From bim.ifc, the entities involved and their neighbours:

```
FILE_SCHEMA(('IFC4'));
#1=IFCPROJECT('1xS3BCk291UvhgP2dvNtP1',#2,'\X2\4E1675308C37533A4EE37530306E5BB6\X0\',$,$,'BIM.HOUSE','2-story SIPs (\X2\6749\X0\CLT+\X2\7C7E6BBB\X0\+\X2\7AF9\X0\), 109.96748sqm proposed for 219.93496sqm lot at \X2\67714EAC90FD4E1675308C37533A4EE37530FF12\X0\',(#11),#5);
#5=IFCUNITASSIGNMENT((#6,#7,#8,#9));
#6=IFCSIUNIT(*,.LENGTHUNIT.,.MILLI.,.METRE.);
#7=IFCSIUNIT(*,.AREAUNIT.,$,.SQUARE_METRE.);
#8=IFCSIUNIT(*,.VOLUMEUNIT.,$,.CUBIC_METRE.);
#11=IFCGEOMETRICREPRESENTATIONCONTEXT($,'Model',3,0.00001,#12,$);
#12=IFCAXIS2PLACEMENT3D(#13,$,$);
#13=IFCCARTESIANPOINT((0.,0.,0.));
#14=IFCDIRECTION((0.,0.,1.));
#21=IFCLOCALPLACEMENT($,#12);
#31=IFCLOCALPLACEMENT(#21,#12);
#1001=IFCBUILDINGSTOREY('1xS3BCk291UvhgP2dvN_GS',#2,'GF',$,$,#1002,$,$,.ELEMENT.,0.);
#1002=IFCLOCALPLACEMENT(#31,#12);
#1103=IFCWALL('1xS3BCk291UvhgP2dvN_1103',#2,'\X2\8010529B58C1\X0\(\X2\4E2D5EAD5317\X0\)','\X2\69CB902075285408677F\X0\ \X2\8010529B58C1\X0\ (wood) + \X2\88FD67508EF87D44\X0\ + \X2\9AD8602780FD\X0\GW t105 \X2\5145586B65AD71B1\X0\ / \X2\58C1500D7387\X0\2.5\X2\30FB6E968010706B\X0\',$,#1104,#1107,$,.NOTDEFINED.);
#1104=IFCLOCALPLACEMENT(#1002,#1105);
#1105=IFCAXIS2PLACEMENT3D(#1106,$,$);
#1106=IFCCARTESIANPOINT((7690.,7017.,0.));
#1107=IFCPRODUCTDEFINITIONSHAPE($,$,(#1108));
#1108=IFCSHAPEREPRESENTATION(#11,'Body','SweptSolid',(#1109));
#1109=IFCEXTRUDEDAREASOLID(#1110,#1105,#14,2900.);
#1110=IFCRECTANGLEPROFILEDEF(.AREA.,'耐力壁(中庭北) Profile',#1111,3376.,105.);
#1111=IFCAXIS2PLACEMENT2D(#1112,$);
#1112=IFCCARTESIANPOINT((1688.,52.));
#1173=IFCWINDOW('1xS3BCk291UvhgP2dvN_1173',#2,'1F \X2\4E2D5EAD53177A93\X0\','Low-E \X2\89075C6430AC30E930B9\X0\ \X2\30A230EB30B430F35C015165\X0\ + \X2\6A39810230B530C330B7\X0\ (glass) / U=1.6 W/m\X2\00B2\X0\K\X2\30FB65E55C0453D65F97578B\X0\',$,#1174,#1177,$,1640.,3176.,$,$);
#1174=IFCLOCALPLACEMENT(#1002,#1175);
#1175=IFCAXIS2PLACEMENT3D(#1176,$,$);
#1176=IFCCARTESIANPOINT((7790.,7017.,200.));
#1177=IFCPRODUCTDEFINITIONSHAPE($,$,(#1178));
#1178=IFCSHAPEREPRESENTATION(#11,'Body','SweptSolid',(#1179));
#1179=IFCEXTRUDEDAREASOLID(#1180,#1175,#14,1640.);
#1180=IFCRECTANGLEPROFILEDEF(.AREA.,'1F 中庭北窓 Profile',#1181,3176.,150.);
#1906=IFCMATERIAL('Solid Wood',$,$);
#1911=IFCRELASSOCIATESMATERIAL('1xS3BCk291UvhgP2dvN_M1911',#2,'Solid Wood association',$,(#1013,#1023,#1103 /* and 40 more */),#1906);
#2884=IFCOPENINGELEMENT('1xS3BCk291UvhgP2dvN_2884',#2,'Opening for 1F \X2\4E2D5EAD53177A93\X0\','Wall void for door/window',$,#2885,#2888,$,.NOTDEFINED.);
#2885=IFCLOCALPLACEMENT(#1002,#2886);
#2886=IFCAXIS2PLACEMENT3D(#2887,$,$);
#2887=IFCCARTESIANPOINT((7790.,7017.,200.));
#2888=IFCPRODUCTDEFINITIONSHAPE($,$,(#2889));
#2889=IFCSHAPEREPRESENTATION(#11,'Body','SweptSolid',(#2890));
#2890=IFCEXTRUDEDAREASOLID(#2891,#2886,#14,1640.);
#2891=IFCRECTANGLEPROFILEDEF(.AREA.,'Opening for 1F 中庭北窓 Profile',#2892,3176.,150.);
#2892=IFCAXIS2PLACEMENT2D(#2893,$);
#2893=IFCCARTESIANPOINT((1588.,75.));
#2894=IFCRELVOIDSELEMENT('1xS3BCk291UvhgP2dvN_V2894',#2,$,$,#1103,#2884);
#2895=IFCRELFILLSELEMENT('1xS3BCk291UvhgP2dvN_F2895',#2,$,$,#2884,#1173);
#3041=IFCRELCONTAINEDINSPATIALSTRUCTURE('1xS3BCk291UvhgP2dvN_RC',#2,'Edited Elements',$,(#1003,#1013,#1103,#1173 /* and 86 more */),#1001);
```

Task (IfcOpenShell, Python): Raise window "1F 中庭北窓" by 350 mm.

```python
import numpy as np
import ifcopenshell
import ifcopenshell.api.geometry
import ifcopenshell.util.placement
import ifcopenshell.util.unit

model = ifcopenshell.open("bim.ifc")
unit_scale = ifcopenshell.util.unit.calculate_unit_scale(model)

window = model.by_guid("1xS3BCk291UvhgP2dvN_1173")
opening = window.FillsVoids[0].RelatingOpeningElement
dz = 350.0

shift = np.array([0.0, 0.0, dz])
# The window is not placed relative to its opening, so move both.
for product in (opening, window):
    matrix = ifcopenshell.util.placement.get_local_placement(product.ObjectPlacement)
    matrix[:3, 3] += shift
    ifcopenshell.api.geometry.edit_object_placement(model, product=product, matrix=matrix, is_si=False)

print(f"moved by {dz * unit_scale:+.3f} m")

model.write("bim_rev.ifc")
```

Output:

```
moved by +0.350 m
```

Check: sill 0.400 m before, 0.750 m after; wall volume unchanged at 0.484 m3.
